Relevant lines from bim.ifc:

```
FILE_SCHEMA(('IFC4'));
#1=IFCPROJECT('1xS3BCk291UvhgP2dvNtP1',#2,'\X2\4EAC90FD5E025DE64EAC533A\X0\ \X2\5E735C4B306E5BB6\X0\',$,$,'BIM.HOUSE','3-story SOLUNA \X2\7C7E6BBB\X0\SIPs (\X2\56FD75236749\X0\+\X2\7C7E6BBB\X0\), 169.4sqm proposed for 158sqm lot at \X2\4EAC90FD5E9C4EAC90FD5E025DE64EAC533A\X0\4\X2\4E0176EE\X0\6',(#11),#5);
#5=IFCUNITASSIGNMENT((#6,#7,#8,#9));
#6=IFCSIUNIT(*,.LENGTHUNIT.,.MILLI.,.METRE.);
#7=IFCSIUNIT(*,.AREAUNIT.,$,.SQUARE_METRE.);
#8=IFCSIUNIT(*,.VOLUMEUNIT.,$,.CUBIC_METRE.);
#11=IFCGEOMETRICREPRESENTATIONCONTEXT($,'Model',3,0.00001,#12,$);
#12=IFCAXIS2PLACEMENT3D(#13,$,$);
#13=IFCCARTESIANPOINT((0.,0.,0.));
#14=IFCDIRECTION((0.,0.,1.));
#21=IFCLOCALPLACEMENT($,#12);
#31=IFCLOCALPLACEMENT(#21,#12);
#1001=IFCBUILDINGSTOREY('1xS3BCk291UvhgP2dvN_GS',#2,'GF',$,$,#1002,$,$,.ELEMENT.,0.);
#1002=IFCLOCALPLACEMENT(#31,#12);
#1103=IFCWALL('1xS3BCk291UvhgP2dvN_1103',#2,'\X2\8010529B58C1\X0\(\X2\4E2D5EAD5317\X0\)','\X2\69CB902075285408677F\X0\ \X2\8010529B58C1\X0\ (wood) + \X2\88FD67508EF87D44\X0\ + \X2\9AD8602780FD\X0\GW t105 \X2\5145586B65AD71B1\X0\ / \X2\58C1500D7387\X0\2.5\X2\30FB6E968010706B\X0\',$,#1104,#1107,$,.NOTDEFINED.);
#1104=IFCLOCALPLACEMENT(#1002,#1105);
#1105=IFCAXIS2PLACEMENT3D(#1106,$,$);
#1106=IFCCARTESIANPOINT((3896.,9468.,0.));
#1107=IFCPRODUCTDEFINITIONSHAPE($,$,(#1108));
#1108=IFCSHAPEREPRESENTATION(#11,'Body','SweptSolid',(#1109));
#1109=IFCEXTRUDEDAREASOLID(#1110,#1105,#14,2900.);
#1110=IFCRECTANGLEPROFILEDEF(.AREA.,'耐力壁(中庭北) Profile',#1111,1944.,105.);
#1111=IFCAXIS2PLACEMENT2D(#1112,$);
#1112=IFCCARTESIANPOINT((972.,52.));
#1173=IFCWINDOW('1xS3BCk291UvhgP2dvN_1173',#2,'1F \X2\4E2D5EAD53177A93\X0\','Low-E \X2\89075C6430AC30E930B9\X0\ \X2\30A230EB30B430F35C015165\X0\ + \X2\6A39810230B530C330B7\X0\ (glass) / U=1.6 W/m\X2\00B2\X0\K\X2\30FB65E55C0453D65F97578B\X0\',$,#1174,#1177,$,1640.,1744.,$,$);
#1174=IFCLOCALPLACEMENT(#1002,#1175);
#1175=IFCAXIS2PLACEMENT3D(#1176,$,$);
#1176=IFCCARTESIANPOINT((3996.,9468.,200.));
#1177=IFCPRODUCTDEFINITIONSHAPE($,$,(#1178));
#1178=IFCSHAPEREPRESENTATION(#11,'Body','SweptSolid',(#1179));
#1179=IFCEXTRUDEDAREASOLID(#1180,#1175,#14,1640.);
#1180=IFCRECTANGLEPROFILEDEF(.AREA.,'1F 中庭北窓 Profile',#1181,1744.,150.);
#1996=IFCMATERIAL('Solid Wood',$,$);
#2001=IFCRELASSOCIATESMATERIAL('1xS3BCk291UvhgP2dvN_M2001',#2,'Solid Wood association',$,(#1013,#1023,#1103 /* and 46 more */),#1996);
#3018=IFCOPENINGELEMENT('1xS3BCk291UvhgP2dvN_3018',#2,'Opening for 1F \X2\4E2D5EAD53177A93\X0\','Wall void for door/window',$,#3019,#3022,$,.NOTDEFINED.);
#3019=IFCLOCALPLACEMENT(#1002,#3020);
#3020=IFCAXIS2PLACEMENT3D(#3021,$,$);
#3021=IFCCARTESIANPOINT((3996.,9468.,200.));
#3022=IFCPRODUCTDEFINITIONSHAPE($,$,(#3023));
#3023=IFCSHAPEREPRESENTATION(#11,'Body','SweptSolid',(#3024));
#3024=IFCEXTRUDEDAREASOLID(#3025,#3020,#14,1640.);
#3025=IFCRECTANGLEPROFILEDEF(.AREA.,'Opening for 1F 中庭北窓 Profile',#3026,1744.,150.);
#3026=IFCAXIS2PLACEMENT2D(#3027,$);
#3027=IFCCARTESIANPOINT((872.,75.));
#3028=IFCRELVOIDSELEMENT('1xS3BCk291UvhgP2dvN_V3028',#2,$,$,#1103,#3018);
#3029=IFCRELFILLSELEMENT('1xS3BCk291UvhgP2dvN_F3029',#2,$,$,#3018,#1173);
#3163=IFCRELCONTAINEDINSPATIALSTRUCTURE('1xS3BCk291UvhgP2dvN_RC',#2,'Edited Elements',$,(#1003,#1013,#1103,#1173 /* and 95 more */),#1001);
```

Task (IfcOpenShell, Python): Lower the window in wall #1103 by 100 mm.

```python
import numpy as np
import ifcopenshell
import ifcopenshell.api.geometry
import ifcopenshell.util.placement
import ifcopenshell.util.unit

model = ifcopenshell.open("bim.ifc")
unit_scale = ifcopenshell.util.unit.calculate_unit_scale(model)

window = model.by_guid("1xS3BCk291UvhgP2dvN_1173")
opening = window.FillsVoids[0].RelatingOpeningElement
dz = -100.0

shift = np.array([0.0, 0.0, dz])
# The window is not placed relative to its opening, so move both.
for product in (opening, window):
    matrix = ifcopenshell.util.placement.get_local_placement(product.ObjectPlacement)
    matrix[:3, 3] += shift
    ifcopenshell.api.geometry.edit_object_placement(model, product=product, matrix=matrix, is_si=False)

print(f"moved by {dz * unit_scale:+.3f} m")

model.write("bim_v2.ifc")
```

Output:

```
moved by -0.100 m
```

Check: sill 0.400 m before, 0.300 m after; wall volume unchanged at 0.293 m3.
